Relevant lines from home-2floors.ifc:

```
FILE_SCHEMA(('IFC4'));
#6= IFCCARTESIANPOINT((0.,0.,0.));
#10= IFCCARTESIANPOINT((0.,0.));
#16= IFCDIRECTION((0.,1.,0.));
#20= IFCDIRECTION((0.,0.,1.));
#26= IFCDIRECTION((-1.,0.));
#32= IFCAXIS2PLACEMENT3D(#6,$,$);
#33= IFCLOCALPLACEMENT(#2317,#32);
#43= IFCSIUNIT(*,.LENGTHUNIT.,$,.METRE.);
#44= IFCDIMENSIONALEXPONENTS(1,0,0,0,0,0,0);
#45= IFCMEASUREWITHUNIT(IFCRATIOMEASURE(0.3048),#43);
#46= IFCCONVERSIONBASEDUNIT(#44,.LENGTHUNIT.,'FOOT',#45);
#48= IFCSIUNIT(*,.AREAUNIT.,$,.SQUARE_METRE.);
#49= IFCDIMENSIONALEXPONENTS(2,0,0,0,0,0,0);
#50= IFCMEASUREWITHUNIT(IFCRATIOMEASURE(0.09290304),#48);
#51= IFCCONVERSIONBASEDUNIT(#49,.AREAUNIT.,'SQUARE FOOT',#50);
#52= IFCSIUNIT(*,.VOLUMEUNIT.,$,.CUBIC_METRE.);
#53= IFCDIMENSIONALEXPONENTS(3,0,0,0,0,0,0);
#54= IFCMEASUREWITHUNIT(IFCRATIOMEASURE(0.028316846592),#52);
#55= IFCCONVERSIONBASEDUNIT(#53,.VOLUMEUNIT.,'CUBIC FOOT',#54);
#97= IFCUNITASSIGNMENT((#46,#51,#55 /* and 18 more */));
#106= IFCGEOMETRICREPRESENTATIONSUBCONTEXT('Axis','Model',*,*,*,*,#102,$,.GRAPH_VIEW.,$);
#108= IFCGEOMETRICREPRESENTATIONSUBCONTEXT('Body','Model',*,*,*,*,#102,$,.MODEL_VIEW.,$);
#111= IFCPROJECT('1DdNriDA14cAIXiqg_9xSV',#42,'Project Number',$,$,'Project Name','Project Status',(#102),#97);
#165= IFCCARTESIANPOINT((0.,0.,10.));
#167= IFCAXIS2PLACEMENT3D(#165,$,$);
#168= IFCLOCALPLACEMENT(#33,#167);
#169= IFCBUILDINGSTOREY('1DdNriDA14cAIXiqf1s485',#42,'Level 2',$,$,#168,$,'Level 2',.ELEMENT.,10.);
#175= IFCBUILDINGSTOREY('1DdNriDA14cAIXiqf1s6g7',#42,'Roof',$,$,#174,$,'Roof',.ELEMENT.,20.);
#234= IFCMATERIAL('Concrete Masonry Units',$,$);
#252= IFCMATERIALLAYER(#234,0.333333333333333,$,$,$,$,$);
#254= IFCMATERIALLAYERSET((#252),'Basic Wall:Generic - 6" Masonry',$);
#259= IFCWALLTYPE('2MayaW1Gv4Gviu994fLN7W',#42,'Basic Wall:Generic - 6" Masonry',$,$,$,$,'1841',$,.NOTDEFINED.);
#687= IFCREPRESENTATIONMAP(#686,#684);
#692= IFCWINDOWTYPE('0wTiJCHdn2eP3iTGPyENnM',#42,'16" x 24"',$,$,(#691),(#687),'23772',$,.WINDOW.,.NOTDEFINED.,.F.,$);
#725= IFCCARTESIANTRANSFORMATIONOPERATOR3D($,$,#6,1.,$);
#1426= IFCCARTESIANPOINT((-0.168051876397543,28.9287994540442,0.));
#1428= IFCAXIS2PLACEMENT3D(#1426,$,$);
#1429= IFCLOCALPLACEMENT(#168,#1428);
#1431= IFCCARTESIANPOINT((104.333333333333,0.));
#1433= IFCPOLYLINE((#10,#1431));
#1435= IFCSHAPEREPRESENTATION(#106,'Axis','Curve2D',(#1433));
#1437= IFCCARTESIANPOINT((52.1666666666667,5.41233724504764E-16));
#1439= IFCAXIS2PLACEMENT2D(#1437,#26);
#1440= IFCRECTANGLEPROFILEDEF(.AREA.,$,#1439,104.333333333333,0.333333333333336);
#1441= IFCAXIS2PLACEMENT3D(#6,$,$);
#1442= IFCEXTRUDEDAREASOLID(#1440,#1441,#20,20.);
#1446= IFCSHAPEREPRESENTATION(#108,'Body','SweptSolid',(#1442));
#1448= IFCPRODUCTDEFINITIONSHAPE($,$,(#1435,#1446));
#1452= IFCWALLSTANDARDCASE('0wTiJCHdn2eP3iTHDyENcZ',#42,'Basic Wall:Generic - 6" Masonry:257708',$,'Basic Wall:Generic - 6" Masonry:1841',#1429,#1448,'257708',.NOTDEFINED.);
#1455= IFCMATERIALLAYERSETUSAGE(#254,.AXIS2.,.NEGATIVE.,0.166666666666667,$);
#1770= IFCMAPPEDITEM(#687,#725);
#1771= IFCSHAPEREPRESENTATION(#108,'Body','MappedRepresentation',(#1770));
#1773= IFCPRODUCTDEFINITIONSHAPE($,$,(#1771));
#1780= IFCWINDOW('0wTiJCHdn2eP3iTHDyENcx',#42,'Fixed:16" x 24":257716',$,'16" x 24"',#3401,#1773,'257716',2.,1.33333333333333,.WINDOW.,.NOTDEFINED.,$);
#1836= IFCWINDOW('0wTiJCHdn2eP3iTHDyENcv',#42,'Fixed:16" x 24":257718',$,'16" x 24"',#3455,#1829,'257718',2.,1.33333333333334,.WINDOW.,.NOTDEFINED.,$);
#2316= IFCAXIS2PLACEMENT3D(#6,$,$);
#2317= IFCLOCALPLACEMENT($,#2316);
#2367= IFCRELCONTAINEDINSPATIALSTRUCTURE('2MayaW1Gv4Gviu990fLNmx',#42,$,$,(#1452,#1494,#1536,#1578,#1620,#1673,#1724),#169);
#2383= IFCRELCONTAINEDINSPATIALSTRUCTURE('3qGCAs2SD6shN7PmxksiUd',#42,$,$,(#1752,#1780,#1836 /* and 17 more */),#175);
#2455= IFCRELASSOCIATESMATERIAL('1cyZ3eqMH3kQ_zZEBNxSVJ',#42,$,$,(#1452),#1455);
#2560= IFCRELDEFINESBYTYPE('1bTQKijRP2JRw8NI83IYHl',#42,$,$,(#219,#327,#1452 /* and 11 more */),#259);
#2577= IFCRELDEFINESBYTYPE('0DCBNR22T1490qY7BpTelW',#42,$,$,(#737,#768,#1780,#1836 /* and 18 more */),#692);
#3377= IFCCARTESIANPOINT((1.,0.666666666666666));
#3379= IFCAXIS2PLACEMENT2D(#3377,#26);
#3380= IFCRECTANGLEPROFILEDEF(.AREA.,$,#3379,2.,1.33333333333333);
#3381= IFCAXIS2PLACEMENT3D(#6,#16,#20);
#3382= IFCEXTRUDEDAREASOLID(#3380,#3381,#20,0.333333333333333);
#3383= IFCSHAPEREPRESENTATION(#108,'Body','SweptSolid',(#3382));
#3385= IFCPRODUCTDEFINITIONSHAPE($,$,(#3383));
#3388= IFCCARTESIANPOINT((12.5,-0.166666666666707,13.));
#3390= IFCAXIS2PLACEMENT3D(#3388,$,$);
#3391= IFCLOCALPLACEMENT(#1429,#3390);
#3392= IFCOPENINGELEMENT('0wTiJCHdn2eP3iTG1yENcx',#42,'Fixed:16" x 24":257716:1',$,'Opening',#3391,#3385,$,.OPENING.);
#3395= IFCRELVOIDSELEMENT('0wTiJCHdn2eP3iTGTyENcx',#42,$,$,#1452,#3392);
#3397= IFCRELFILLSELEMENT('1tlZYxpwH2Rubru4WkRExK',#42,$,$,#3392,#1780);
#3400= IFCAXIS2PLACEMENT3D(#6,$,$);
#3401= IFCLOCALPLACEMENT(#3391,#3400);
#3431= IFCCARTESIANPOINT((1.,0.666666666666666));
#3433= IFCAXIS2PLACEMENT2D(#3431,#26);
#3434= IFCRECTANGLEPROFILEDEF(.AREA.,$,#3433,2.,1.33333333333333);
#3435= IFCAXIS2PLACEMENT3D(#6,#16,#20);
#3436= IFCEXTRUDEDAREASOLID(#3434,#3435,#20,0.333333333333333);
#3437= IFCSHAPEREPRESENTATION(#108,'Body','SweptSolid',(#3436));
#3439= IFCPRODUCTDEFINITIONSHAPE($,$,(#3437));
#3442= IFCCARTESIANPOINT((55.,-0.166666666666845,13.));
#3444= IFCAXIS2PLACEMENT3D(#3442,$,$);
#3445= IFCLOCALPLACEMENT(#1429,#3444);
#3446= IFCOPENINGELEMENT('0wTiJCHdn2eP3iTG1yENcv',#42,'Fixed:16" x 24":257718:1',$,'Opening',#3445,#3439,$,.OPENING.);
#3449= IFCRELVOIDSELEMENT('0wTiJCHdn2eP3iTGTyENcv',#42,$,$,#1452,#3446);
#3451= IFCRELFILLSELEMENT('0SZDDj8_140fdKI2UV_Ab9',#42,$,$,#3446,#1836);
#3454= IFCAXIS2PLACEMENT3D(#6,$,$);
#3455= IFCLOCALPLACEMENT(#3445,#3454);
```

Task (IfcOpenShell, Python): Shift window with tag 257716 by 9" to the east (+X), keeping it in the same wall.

```python
import ifcopenshell
import ifcopenshell.api.geometry
import ifcopenshell.util.placement
import ifcopenshell.util.unit

model = ifcopenshell.open("home-2floors.ifc")
unit_scale = ifcopenshell.util.unit.calculate_unit_scale(model)

window = model.by_id(1780)
opening = window.FillsVoids[0].RelatingOpeningElement
wall = opening.VoidsElements[0].RelatingBuildingElement

wall_matrix = ifcopenshell.util.placement.get_local_placement(wall.ObjectPlacement)
shift = wall_matrix[:3, 0] * 9 * 0.0254 / unit_scale
before = ifcopenshell.util.placement.get_local_placement(window.ObjectPlacement)[:3, 3].copy()

# The window is placed relative to its opening, so it follows when the opening moves.
matrix = ifcopenshell.util.placement.get_local_placement(opening.ObjectPlacement)
matrix[:3, 3] += shift
ifcopenshell.api.geometry.edit_object_placement(
    model, product=opening, matrix=matrix, is_si=False, should_transform_children=True
)

after = ifcopenshell.util.placement.get_local_placement(window.ObjectPlacement)[:3, 3]
print("window moved by", (after - before).round(3) + 0.0)

model.write("home-2floors_rev.ifc")
```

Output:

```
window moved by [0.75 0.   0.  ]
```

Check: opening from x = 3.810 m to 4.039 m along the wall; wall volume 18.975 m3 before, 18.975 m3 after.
